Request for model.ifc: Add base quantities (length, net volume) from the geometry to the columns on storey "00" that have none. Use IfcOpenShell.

First a look at what the model holds.

```python
import ifcopenshell
import ifcopenshell.util.element
import ifcopenshell.util.unit

model = ifcopenshell.open("model.ifc")
print(model.schema)
for unit_type in ("LENGTHUNIT", "AREAUNIT", "VOLUMEUNIT"):
    print(unit_type, ifcopenshell.util.unit.calculate_unit_scale(model, unit_type))
storey = next(s for s in model.by_type("IfcBuildingStorey") if s.Name == "00")
columns = [e for e in ifcopenshell.util.element.get_decomposition(storey) if e.is_a("IfcColumn")]
for e in sorted(columns, key=lambda e: e.id()):
    print(e.id(), e.is_a(), e.Name, list(ifcopenshell.util.element.get_psets(e, qtos_only=True)), sep=" | ")
```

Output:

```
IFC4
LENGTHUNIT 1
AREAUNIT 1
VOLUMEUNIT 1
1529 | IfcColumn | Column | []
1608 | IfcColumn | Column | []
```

```python
import ifcopenshell
import ifcopenshell.api.pset
import ifcopenshell.geom
import ifcopenshell.util.element
import ifcopenshell.util.shape
import ifcopenshell.util.unit

model = ifcopenshell.open("model.ifc")
unit_scale = ifcopenshell.util.unit.calculate_unit_scale(model)
volume_scale = ifcopenshell.util.unit.calculate_unit_scale(model, "VOLUMEUNIT")
settings = ifcopenshell.geom.settings()

storey = next(s for s in model.by_type("IfcBuildingStorey") if s.Name == "00")
columns = [e for e in ifcopenshell.util.element.get_decomposition(storey) if e.is_a("IfcColumn")]

for e in sorted(columns, key=lambda e: e.id()):
    if ifcopenshell.util.element.get_psets(e, qtos_only=True, should_inherit=False):
        continue
    # Geometry comes back in metres, in the element's own axes.
    shape = ifcopenshell.geom.create_shape(settings, e)
    values = {
        "Length": ifcopenshell.util.shape.get_z(shape.geometry) / unit_scale,
        "NetVolume": ifcopenshell.util.shape.get_volume(shape.geometry) / volume_scale,
    }
    qto = ifcopenshell.api.pset.add_qto(model, product=e, name="Qto_ColumnBaseQuantities")
    ifcopenshell.api.pset.edit_qto(model, qto=qto, properties=values)
    print(e.id(), {k: round(v, 3) for k, v in values.items()})

model.write("model_updated.ifc")
```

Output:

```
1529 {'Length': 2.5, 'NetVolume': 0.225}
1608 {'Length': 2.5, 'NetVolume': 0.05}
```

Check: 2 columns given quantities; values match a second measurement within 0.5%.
